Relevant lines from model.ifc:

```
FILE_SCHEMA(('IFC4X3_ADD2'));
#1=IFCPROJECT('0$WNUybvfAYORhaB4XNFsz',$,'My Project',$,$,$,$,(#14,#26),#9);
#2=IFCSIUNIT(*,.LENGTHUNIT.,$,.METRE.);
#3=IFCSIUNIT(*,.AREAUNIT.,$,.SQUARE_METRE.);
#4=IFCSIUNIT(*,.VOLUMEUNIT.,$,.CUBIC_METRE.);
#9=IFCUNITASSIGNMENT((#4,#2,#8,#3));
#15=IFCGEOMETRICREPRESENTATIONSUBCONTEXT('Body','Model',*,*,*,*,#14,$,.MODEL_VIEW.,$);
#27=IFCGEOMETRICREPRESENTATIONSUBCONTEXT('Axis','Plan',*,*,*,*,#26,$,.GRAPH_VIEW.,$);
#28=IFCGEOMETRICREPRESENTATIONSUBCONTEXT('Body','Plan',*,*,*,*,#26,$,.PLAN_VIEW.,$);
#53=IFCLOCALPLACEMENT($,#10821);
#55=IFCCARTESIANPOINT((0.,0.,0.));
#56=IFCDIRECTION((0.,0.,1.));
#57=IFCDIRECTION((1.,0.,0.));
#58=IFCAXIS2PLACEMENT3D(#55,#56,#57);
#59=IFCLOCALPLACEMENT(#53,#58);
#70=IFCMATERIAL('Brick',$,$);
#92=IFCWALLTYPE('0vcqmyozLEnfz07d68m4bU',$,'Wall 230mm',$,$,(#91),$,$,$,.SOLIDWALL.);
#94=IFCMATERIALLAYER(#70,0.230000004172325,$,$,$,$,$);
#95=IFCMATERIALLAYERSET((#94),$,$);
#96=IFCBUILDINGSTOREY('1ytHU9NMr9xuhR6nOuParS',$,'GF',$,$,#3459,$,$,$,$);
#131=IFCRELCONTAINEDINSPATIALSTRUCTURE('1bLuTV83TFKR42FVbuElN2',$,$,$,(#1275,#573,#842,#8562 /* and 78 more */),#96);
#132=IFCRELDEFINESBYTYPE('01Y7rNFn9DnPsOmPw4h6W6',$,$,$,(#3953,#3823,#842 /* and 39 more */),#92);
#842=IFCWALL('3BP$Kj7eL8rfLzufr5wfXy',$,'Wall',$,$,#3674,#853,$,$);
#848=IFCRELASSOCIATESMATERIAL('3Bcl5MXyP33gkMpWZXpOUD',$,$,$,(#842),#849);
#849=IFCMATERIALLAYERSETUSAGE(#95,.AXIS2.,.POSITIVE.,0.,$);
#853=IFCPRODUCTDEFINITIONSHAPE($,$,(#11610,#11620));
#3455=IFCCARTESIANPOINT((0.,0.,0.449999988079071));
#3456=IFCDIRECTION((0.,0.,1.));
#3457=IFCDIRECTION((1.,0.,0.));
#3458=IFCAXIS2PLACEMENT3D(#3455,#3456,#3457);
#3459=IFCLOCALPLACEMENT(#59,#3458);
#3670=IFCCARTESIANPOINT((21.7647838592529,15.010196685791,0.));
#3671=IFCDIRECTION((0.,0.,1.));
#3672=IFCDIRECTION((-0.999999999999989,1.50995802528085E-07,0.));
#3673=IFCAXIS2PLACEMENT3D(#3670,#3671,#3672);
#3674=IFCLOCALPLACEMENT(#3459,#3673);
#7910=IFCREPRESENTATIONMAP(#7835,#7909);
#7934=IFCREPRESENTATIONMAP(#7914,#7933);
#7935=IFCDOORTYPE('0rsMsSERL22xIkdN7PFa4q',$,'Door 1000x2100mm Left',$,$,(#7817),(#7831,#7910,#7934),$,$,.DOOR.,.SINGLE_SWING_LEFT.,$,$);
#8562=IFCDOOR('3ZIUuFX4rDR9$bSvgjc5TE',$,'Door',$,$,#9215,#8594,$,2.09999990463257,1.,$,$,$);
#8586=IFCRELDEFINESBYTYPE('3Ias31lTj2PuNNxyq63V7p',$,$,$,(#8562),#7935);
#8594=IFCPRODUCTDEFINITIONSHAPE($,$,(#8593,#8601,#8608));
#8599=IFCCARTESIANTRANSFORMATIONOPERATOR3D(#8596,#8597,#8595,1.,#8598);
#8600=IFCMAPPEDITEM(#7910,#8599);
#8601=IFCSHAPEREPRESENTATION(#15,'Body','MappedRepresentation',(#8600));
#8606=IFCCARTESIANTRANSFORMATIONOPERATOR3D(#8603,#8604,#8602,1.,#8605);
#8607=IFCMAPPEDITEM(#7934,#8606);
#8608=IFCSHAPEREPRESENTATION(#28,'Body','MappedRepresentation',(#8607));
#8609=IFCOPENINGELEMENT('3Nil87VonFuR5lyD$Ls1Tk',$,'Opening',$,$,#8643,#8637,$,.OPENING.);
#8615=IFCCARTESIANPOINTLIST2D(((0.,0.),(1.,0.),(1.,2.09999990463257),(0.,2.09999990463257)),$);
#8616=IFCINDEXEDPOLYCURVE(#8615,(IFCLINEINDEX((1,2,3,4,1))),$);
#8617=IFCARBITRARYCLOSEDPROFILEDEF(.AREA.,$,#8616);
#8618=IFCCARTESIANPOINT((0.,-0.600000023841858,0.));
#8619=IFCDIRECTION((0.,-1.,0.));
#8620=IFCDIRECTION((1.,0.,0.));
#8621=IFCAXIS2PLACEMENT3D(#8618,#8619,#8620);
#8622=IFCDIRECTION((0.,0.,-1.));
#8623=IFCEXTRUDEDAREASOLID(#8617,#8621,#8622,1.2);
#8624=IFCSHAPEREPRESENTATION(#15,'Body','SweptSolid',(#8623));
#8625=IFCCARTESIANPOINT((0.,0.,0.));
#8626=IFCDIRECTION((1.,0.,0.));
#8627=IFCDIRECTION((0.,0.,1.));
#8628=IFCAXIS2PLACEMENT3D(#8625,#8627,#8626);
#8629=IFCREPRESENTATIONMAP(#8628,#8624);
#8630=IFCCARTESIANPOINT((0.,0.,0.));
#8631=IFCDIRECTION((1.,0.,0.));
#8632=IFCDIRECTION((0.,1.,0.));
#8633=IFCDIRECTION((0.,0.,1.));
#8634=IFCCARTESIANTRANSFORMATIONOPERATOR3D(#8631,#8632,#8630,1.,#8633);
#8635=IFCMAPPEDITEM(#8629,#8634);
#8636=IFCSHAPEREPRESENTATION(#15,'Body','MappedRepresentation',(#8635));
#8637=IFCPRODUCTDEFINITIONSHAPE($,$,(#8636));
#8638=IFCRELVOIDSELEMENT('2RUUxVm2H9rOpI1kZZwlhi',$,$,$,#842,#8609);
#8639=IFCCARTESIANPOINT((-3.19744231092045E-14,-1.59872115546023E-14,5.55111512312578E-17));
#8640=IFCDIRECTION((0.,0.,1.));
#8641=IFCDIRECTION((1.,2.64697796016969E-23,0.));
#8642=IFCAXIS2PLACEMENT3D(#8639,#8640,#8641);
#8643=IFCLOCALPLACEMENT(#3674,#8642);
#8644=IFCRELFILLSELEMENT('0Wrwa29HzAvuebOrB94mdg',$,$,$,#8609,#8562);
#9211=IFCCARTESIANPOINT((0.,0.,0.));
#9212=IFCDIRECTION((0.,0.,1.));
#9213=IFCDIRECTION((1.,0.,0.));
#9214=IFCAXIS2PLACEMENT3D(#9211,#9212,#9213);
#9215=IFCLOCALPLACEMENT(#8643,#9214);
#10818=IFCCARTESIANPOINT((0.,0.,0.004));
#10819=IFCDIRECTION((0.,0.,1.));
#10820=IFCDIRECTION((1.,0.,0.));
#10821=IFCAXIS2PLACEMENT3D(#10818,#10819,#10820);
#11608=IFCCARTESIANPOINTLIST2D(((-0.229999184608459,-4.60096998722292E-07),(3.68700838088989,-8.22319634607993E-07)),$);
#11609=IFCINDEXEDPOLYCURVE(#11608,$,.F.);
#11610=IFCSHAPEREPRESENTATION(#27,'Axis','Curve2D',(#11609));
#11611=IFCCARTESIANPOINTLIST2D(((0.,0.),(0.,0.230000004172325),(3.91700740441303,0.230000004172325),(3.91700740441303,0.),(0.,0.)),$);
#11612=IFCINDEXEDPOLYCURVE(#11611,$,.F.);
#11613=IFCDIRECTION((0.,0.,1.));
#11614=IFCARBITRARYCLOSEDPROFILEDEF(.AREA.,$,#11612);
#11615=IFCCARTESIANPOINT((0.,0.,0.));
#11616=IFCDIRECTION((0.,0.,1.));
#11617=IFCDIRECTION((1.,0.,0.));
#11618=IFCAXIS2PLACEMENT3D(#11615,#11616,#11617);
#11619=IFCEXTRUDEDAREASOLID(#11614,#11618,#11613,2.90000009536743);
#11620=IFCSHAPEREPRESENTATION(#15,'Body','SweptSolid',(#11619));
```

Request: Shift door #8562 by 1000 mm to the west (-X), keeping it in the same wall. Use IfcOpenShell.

```python
import ifcopenshell
import ifcopenshell.api.geometry
import ifcopenshell.util.placement
import ifcopenshell.util.unit

model = ifcopenshell.open("model.ifc")
unit_scale = ifcopenshell.util.unit.calculate_unit_scale(model)

door = model.by_id(8562)
opening = door.FillsVoids[0].RelatingOpeningElement
wall = opening.VoidsElements[0].RelatingBuildingElement

wall_matrix = ifcopenshell.util.placement.get_local_placement(wall.ObjectPlacement)
shift = wall_matrix[:3, 0] * 1 / unit_scale
before = ifcopenshell.util.placement.get_local_placement(door.ObjectPlacement)[:3, 3].copy()

# The door is placed relative to its opening, so it follows when the opening moves.
matrix = ifcopenshell.util.placement.get_local_placement(opening.ObjectPlacement)
matrix[:3, 3] += shift
ifcopenshell.api.geometry.edit_object_placement(
    model, product=opening, matrix=matrix, is_si=False, should_transform_children=True
)

after = ifcopenshell.util.placement.get_local_placement(door.ObjectPlacement)[:3, 3]
print("door moved by", (after - before).round(3) + 0.0)

model.write("model-out.ifc")
```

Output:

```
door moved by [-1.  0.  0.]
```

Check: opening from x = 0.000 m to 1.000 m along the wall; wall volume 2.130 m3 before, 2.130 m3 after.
